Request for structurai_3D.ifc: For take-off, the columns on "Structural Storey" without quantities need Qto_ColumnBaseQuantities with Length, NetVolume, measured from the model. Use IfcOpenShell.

First a look at what the model holds.

```python
import ifcopenshell
import ifcopenshell.util.element
import ifcopenshell.util.unit

model = ifcopenshell.open("structurai_3D.ifc")
print(model.schema)
for unit_type in ("LENGTHUNIT", "AREAUNIT", "VOLUMEUNIT"):
    print(unit_type, ifcopenshell.util.unit.calculate_unit_scale(model, unit_type))
storey = next(s for s in model.by_type("IfcBuildingStorey") if s.Name == "Structural Storey")
columns = [e for e in ifcopenshell.util.element.get_decomposition(storey) if e.is_a("IfcColumn")]
for e in sorted(columns, key=lambda e: e.id()):
    print(e.id(), e.is_a(), e.Name, list(ifcopenshell.util.element.get_psets(e, qtos_only=True)), sep=" | ")
```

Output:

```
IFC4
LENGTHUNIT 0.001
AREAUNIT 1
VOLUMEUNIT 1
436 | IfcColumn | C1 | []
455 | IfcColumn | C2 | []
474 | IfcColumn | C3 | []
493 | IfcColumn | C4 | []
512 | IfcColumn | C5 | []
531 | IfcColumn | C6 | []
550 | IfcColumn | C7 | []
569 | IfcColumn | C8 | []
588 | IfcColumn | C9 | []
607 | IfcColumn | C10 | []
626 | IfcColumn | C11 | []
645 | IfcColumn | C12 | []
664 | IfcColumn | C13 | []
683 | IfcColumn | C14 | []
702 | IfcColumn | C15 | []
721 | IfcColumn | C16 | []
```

```python
import ifcopenshell
import ifcopenshell.api.pset
import ifcopenshell.geom
import ifcopenshell.util.element
import ifcopenshell.util.shape
import ifcopenshell.util.unit

model = ifcopenshell.open("structurai_3D.ifc")
unit_scale = ifcopenshell.util.unit.calculate_unit_scale(model)
volume_scale = ifcopenshell.util.unit.calculate_unit_scale(model, "VOLUMEUNIT")
settings = ifcopenshell.geom.settings()

storey = next(s for s in model.by_type("IfcBuildingStorey") if s.Name == "Structural Storey")
columns = [e for e in ifcopenshell.util.element.get_decomposition(storey) if e.is_a("IfcColumn")]

for e in sorted(columns, key=lambda e: e.id()):
    if ifcopenshell.util.element.get_psets(e, qtos_only=True, should_inherit=False):
        continue
    # Geometry comes back in metres, in the element's own axes.
    shape = ifcopenshell.geom.create_shape(settings, e)
    values = {
        "Length": ifcopenshell.util.shape.get_z(shape.geometry) / unit_scale,
        "NetVolume": ifcopenshell.util.shape.get_volume(shape.geometry) / volume_scale,
    }
    qto = ifcopenshell.api.pset.add_qto(model, product=e, name="Qto_ColumnBaseQuantities")
    ifcopenshell.api.pset.edit_qto(model, qto=qto, properties=values)
    print(e.id(), {k: round(v, 3) for k, v in values.items()})

model.write("structurai_3D_v2.ifc")
```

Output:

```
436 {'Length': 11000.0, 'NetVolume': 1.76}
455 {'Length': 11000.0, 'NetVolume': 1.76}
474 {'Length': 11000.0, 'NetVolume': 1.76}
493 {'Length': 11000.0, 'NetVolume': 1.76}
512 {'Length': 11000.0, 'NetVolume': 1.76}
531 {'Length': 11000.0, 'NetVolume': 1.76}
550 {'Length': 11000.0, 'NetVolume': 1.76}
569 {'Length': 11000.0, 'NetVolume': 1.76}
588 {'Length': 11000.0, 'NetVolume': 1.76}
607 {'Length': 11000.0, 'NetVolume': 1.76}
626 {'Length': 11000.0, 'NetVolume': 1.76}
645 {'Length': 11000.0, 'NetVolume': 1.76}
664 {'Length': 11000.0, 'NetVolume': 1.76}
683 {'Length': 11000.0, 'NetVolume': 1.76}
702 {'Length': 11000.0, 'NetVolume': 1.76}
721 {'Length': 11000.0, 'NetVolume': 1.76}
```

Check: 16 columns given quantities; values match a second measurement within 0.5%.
